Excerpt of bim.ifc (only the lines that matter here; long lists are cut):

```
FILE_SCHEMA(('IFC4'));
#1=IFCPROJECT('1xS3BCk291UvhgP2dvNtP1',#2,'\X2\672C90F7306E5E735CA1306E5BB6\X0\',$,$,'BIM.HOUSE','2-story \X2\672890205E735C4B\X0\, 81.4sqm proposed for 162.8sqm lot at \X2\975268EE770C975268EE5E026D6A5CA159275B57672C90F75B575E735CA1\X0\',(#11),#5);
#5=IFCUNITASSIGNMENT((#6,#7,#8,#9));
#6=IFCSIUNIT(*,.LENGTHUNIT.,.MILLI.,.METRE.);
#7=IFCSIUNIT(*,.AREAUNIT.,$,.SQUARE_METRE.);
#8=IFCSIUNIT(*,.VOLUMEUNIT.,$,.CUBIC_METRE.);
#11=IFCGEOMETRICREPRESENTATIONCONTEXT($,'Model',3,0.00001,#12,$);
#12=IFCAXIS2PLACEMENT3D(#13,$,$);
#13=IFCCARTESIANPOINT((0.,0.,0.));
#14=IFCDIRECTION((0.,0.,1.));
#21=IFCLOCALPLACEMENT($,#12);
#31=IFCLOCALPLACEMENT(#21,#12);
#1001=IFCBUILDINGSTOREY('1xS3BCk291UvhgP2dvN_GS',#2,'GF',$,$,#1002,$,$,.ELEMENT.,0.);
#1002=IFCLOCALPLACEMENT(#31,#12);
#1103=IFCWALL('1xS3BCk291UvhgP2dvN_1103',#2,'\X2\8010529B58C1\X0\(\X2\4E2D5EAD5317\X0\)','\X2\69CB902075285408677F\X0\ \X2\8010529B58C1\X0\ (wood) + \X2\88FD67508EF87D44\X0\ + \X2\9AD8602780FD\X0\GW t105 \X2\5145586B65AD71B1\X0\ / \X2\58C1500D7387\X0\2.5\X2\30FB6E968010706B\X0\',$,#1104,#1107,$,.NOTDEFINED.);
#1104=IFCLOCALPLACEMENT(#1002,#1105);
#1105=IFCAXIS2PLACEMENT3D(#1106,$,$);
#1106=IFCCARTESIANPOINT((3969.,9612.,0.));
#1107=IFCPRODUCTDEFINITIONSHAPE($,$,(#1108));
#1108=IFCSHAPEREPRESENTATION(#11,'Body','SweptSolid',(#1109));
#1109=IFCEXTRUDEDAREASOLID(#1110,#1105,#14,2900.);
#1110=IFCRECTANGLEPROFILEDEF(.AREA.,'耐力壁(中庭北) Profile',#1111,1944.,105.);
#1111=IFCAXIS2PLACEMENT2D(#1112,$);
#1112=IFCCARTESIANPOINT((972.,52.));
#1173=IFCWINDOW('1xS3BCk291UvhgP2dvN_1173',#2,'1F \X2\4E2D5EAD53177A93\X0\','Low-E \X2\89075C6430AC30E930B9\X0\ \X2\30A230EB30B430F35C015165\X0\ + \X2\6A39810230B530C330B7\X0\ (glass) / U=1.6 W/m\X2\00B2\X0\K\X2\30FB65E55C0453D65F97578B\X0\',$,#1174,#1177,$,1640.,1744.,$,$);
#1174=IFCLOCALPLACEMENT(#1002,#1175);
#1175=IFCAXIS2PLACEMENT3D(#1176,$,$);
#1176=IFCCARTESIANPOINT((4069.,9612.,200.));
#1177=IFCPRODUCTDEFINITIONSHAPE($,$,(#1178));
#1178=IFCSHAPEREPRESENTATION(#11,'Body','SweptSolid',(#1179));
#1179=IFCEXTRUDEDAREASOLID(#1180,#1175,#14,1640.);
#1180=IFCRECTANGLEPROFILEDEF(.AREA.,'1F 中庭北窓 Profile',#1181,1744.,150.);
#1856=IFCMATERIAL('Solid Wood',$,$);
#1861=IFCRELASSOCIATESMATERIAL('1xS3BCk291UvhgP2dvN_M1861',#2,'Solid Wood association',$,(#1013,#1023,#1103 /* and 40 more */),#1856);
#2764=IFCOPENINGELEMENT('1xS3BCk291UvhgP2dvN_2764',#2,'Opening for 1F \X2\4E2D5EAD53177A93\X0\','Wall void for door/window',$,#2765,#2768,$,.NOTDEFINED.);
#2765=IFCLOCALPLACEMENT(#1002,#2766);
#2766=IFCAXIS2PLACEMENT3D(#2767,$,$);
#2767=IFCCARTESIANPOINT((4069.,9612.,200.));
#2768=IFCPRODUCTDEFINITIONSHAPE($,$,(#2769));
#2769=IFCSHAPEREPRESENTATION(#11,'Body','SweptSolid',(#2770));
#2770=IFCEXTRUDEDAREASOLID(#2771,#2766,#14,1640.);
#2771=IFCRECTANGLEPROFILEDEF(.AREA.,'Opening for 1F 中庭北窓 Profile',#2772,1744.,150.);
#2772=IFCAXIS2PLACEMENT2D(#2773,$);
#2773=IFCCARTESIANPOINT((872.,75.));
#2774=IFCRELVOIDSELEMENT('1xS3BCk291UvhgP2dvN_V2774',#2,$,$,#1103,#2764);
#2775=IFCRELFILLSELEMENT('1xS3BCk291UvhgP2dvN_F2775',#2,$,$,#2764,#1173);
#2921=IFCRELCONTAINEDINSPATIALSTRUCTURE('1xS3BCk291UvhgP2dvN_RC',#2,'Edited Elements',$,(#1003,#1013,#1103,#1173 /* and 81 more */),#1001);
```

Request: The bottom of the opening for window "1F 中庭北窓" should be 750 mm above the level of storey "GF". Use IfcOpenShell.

```python
import numpy as np
import ifcopenshell
import ifcopenshell.api.geometry
import ifcopenshell.geom
import ifcopenshell.util.element
import ifcopenshell.util.placement
import ifcopenshell.util.shape
import ifcopenshell.util.unit

model = ifcopenshell.open("bim.ifc")
unit_scale = ifcopenshell.util.unit.calculate_unit_scale(model)

window = model.by_guid("1xS3BCk291UvhgP2dvN_1173")
opening = window.FillsVoids[0].RelatingOpeningElement
storey = ifcopenshell.util.element.get_container(window, ifc_class="IfcBuildingStorey")
level = ifcopenshell.util.placement.get_local_placement(storey.ObjectPlacement)[2, 3]

# The opening's origin need not be at the sill, so measure its lowest point.
shape = ifcopenshell.geom.create_shape(ifcopenshell.geom.settings(), opening)
bottom = ifcopenshell.util.shape.get_shape_bottom_elevation(shape, shape.geometry) / unit_scale
dz = level + 0.75 / unit_scale - bottom

shift = np.array([0.0, 0.0, dz])
# The window is not placed relative to its opening, so move both.
for product in (opening, window):
    matrix = ifcopenshell.util.placement.get_local_placement(product.ObjectPlacement)
    matrix[:3, 3] += shift
    ifcopenshell.api.geometry.edit_object_placement(model, product=product, matrix=matrix, is_si=False)

print(f"moved by {dz * unit_scale:+.3f} m")

model.write("bim_v2.ifc")
```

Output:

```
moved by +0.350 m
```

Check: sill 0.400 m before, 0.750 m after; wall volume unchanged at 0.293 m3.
